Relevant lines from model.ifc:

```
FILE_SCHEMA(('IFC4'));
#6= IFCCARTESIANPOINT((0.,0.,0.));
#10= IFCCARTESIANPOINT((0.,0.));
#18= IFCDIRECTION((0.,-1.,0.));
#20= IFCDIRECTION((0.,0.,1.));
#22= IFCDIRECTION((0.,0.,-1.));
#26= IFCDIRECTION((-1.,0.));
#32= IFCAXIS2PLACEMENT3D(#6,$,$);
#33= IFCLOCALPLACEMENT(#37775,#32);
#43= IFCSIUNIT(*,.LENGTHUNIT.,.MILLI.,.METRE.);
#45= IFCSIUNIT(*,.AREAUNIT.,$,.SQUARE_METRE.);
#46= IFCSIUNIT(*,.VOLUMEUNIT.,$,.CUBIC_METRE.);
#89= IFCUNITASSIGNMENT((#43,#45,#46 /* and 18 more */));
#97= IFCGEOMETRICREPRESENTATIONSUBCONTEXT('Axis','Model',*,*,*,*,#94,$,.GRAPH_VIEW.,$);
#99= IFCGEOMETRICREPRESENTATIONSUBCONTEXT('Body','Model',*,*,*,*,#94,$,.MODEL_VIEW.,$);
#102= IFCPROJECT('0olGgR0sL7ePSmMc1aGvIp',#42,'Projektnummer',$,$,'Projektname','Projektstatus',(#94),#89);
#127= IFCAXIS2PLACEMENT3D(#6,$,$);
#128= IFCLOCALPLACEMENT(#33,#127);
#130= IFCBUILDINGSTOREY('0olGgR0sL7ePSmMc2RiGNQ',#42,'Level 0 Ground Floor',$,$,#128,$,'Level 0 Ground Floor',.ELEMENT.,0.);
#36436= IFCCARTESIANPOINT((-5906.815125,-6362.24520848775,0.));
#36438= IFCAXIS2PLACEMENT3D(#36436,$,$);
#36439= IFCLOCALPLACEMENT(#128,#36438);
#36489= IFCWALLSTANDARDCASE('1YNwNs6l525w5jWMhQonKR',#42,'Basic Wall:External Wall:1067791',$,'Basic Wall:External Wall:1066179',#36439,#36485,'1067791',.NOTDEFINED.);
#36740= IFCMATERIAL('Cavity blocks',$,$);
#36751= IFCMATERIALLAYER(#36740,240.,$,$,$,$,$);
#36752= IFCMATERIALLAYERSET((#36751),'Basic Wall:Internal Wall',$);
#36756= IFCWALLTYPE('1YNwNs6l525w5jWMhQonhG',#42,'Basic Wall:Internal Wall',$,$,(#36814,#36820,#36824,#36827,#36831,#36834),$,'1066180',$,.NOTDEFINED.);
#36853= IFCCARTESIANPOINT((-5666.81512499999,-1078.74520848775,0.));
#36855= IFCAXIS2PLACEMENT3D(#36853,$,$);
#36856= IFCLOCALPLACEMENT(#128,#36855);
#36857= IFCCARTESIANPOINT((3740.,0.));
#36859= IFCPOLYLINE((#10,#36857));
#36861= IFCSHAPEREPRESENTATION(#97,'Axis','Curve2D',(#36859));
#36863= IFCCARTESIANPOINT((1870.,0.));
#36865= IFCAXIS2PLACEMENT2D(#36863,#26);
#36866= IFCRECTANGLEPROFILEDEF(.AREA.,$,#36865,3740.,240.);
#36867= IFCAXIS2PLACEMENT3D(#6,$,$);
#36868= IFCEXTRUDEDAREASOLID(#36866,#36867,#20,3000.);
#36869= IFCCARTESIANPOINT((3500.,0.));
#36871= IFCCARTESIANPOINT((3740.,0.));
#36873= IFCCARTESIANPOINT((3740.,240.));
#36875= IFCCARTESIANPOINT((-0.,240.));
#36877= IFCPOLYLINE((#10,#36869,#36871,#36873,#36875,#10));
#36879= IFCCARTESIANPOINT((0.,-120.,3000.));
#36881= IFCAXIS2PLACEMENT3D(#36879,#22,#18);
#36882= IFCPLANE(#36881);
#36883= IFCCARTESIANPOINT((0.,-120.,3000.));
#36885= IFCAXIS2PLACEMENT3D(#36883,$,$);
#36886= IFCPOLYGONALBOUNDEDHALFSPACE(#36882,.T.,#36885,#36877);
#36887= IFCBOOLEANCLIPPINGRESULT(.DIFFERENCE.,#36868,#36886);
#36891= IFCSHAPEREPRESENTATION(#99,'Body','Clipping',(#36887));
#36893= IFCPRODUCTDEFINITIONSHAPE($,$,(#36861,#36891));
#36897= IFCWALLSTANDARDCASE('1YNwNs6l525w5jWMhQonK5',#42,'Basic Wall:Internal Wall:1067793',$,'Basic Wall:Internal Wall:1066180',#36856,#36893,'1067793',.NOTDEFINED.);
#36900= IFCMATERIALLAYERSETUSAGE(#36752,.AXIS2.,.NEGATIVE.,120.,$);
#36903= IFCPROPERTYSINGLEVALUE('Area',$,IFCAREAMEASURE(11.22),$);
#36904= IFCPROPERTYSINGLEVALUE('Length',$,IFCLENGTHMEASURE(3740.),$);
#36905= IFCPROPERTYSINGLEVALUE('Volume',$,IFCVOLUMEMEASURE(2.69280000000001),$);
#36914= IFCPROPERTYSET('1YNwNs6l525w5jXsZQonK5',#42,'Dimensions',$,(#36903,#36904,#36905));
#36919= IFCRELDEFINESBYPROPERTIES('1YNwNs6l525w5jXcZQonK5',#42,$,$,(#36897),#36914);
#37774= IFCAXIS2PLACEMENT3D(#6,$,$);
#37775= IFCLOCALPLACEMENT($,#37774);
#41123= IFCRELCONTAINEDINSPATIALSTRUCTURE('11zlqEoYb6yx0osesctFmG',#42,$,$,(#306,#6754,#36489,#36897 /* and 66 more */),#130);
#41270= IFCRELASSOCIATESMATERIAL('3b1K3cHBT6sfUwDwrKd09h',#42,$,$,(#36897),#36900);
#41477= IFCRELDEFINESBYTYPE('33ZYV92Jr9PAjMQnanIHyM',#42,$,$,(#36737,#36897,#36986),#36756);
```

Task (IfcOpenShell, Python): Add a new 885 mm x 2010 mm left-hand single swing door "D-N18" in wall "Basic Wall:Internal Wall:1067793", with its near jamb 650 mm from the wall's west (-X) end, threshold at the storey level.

```python
import numpy as np
import ifcopenshell
import ifcopenshell.api.feature
import ifcopenshell.api.geometry
import ifcopenshell.api.pset
import ifcopenshell.api.root
import ifcopenshell.api.spatial
import ifcopenshell.geom
import ifcopenshell.util.element
import ifcopenshell.util.placement
import ifcopenshell.util.representation
import ifcopenshell.util.shape
import ifcopenshell.util.unit

model = ifcopenshell.open("model.ifc")
unit_scale = ifcopenshell.util.unit.calculate_unit_scale(model)
area_scale = ifcopenshell.util.unit.calculate_unit_scale(model, "AREAUNIT")
volume_scale = ifcopenshell.util.unit.calculate_unit_scale(model, "VOLUMEUNIT")
settings = ifcopenshell.geom.settings()


def volume(element):
    """Net volume in cubic metres, openings subtracted."""
    shape = ifcopenshell.geom.create_shape(settings, element)
    return ifcopenshell.util.shape.get_volume(shape.geometry)


wall = model.by_guid("1YNwNs6l525w5jWMhQonK5")
storey = ifcopenshell.util.element.get_container(wall, ifc_class="IfcBuildingStorey")
context = ifcopenshell.util.representation.get_context(model, "Model", "Body", "MODEL_VIEW")
before = volume(wall)

width, height, from_end, sill = 0.885, 2.01, 0.65, 0.0  # metres

# The wall runs along its own X axis, and the end named is its -X end.
wall_shape = ifcopenshell.geom.create_shape(settings, wall)
x, y, z = ifcopenshell.util.shape.get_vertices(wall_shape.geometry).T
start = x.min() + from_end
face, thickness = float(y.min()), float(y.max() - y.min())
wall_matrix = ifcopenshell.util.placement.get_local_placement(wall.ObjectPlacement)
level = ifcopenshell.util.placement.get_local_placement(storey.ObjectPlacement)[2, 3]


def in_wall(x, y):
    """Placement at x, y metres in the wall's axes, at sill height."""
    matrix = wall_matrix.copy()
    matrix[:, 3] = wall_matrix @ np.array([x / unit_scale, y / unit_scale, 0.0, 1.0])
    matrix[2, 3] = level + sill / unit_scale
    return matrix


# Opening: a box that overshoots both wall faces by 50 mm.
opening = ifcopenshell.api.root.create_entity(model, ifc_class="IfcOpeningElement", predefined_type="OPENING")
box = ifcopenshell.api.geometry.add_wall_representation(
    model, context=context, length=width, height=height, thickness=thickness + 0.1
)
ifcopenshell.api.geometry.assign_representation(model, product=opening, representation=box)
ifcopenshell.api.geometry.edit_object_placement(model, product=opening, matrix=in_wall(start, face - 0.05), is_si=False)
ifcopenshell.api.feature.add_feature(model, feature=opening, element=wall)

door = ifcopenshell.api.root.create_entity(model, ifc_class="IfcDoor", name="D-N18", predefined_type="DOOR")
door.OverallWidth, door.OverallHeight = width / unit_scale, height / unit_scale
door.OperationType = "SINGLE_SWING_LEFT"
body = ifcopenshell.api.geometry.add_door_representation(
    model,
    context=context,
    overall_width=door.OverallWidth,
    overall_height=door.OverallHeight,
    operation_type="SINGLE_SWING_LEFT",
    lining_properties={"LiningDepth": thickness / unit_scale, "ThresholdDepth": thickness / unit_scale},
)
ifcopenshell.api.geometry.assign_representation(model, product=door, representation=body)
ifcopenshell.api.spatial.assign_container(model, products=[door], relating_structure=storey)
ifcopenshell.api.feature.add_filling(model, opening=opening, element=door)

# The lining spans the wall, so the door starts at the wall face.
ifcopenshell.api.geometry.edit_object_placement(model, product=door, matrix=in_wall(start, face), is_si=False)

after = volume(wall)

# Update the wall's stored quantities.
pset = model.by_id(ifcopenshell.util.element.get_pset(wall, "Dimensions", should_inherit=False)["id"])
ifcopenshell.api.pset.edit_pset(model, pset=pset, properties={
    "Area": model.create_entity("IfcAreaMeasure", after / thickness / area_scale),
    "Volume": model.create_entity("IfcVolumeMeasure", after / volume_scale),
})

print(f"wall volume {before:.3f} -> {after:.3f} m3")

model.write("model_edited.ifc")
```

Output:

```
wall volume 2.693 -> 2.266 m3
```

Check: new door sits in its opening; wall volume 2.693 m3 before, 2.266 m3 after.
